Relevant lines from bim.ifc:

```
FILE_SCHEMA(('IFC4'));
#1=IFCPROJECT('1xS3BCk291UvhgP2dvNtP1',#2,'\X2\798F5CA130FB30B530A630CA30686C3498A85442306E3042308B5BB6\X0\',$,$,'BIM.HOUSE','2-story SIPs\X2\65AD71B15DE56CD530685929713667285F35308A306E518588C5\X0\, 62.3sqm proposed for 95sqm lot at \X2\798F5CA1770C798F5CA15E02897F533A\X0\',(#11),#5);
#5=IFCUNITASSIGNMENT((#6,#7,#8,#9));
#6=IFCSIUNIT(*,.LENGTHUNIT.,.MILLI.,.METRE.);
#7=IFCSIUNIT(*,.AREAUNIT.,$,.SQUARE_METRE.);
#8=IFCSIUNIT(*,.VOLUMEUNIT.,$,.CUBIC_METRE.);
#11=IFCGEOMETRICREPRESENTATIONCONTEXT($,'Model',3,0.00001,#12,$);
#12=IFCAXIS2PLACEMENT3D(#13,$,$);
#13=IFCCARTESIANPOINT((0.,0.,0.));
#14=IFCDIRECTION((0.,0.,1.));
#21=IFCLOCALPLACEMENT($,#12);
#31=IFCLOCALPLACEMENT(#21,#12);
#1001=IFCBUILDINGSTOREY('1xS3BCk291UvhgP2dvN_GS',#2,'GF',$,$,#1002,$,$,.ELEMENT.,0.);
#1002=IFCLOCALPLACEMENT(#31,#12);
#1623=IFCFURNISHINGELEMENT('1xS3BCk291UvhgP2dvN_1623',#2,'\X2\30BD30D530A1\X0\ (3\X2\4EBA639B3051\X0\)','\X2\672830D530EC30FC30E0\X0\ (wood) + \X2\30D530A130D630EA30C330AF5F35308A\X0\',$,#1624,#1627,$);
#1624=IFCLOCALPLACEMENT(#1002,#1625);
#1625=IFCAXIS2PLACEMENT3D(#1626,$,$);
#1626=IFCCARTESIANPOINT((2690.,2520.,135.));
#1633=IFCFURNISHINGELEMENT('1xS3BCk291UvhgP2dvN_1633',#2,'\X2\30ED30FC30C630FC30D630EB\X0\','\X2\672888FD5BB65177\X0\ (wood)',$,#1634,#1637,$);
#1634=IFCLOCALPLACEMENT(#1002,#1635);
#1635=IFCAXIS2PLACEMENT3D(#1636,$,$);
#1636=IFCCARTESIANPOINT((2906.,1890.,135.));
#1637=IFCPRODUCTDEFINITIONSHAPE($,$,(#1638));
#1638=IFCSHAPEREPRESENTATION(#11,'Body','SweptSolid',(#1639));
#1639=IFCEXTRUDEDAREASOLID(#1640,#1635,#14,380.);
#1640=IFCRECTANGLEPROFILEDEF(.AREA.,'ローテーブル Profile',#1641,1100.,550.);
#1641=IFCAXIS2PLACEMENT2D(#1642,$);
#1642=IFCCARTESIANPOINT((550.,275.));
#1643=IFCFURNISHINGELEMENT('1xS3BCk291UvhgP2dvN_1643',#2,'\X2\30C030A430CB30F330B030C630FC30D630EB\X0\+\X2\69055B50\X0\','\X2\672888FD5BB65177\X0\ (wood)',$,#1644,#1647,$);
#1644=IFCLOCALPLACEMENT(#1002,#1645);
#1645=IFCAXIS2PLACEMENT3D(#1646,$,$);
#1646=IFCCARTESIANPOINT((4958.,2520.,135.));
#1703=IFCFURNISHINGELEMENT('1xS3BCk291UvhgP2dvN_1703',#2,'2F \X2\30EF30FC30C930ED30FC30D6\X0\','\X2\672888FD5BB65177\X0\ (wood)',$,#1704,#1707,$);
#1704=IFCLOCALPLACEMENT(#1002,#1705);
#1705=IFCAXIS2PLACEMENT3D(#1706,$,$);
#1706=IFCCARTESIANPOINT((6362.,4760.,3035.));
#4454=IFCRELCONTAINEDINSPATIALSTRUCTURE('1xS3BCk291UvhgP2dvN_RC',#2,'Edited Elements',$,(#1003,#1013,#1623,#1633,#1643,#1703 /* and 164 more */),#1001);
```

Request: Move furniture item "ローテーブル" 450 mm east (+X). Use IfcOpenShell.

```python
import ifcopenshell
import ifcopenshell.api.geometry
import ifcopenshell.util.placement
import ifcopenshell.util.unit

model = ifcopenshell.open("bim.ifc")
unit_scale = ifcopenshell.util.unit.calculate_unit_scale(model)

item = model.by_guid("1xS3BCk291UvhgP2dvN_1633")
matrix = ifcopenshell.util.placement.get_local_placement(item.ObjectPlacement)
matrix[0, 3] += 0.45 / unit_scale
ifcopenshell.api.geometry.edit_object_placement(model, product=item, matrix=matrix, is_si=False)

print(ifcopenshell.util.placement.get_local_placement(item.ObjectPlacement).round(3) + 0.0)

model.write("bim_rev.ifc")
```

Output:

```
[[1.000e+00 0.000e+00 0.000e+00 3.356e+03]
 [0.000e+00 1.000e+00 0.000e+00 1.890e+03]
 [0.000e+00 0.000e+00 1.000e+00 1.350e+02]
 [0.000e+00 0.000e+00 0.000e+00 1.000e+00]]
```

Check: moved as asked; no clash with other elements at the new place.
